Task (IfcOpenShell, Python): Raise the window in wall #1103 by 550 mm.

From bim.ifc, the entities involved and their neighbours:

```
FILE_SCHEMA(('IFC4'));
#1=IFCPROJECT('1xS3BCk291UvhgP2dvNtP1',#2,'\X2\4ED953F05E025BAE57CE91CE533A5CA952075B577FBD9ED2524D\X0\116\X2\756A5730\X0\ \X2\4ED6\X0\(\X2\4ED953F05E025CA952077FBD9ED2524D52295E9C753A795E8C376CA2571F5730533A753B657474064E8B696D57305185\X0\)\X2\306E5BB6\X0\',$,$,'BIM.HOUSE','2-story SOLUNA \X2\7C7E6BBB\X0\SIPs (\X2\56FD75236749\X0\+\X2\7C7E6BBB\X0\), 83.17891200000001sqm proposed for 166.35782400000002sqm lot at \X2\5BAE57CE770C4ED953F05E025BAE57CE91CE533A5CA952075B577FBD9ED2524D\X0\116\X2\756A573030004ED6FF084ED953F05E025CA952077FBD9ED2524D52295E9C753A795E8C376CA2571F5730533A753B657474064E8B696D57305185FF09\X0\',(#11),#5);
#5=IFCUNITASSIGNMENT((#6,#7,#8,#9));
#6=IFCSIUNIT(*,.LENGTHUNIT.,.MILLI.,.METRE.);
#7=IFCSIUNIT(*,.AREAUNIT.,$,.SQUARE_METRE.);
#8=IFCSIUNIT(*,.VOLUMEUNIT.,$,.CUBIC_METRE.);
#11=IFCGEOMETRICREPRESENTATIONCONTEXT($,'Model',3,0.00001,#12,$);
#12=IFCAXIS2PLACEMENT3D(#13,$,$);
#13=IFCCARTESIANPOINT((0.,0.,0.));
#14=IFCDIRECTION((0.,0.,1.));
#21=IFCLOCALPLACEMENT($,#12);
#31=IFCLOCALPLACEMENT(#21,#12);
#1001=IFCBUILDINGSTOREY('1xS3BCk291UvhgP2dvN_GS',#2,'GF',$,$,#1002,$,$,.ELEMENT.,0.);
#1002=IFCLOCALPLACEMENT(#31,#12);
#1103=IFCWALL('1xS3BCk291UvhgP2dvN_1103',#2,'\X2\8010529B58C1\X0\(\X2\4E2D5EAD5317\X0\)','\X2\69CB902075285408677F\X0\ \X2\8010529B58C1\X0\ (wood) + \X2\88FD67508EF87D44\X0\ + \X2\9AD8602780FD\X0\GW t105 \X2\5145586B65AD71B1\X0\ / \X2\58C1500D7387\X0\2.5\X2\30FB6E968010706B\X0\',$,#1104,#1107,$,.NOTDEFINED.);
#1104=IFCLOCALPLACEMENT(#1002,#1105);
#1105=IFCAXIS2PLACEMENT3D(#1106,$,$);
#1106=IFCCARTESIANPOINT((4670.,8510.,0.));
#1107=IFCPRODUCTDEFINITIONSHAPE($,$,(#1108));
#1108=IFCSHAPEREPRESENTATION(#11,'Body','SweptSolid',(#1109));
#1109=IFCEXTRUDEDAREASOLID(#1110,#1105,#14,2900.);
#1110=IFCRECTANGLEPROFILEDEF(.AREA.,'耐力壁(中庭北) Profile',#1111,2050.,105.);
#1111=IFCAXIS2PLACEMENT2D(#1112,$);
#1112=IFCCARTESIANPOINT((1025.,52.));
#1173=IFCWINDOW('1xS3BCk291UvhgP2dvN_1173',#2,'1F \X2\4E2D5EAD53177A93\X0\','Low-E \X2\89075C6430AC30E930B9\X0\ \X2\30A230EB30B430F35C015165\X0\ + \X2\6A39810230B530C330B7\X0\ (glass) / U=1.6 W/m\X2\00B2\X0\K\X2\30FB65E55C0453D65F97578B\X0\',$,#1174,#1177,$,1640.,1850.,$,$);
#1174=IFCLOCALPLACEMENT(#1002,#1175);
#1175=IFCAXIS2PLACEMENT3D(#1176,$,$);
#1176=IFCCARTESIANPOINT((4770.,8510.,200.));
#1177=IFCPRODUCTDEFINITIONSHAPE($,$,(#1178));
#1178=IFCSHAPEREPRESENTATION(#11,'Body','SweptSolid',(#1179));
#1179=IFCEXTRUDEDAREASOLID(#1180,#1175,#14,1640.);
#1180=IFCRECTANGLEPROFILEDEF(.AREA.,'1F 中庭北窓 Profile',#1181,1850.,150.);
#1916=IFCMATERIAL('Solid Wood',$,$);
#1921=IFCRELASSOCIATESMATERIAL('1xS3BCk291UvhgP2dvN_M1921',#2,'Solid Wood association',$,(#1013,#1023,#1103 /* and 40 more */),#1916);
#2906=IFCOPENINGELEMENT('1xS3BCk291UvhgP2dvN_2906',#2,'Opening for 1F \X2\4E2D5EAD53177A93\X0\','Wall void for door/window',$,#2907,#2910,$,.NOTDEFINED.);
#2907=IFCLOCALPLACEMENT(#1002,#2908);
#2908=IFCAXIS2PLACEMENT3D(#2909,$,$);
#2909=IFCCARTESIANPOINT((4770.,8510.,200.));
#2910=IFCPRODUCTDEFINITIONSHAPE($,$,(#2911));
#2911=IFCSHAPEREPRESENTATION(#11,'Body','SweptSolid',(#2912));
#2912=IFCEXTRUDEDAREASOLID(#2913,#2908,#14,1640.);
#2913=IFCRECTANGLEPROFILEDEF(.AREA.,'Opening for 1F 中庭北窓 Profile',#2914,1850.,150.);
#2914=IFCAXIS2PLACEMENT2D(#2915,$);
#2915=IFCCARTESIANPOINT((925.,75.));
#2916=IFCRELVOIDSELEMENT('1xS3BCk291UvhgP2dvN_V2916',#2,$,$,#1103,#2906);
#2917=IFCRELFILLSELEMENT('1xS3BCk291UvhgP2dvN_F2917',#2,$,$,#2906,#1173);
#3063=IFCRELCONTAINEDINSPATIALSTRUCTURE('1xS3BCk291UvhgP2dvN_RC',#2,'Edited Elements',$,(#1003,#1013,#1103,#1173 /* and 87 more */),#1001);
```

```python
import numpy as np
import ifcopenshell
import ifcopenshell.api.geometry
import ifcopenshell.util.placement
import ifcopenshell.util.unit

model = ifcopenshell.open("bim.ifc")
unit_scale = ifcopenshell.util.unit.calculate_unit_scale(model)

window = model.by_guid("1xS3BCk291UvhgP2dvN_1173")
opening = window.FillsVoids[0].RelatingOpeningElement
dz = 0.55 / unit_scale

shift = np.array([0.0, 0.0, dz])
# The window is not placed relative to its opening, so move both.
for product in (opening, window):
    matrix = ifcopenshell.util.placement.get_local_placement(product.ObjectPlacement)
    matrix[:3, 3] += shift
    ifcopenshell.api.geometry.edit_object_placement(model, product=product, matrix=matrix, is_si=False)

print(f"moved by {dz * unit_scale:+.3f} m")

model.write("bim_rev.ifc")
```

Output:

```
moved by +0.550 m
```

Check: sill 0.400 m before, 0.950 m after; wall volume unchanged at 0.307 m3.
